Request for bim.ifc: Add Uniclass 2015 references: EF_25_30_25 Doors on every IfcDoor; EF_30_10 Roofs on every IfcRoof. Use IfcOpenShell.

First a look at what the model holds.

```python
import ifcopenshell

model = ifcopenshell.open("bim.ifc")
print(model.schema)
print("classifications:", [c.Name for c in model.by_type("IfcClassification")])
for ifc_class in ("IfcDoor", "IfcRoof", "IfcStair", "IfcWall", "IfcWindow"):
    print(ifc_class, len(model.by_type(ifc_class)))
```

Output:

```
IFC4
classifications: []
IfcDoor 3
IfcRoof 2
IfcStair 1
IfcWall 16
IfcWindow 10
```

```python
import ifcopenshell
import ifcopenshell.api.classification

model = ifcopenshell.open("bim.ifc")

system = ifcopenshell.api.classification.add_classification(model, classification="Uniclass 2015")

codes = {
    "IfcDoor": ("EF_25_30_25", "Doors"),
    "IfcRoof": ("EF_30_10", "Roofs"),
}
for ifc_class, (code, name) in codes.items():
    products = model.by_type(ifc_class)
    ifcopenshell.api.classification.add_reference(
        model, products=products, classification=system, identification=code, name=name
    )
    print(code, len(products))

model.write("bim-out.ifc")
```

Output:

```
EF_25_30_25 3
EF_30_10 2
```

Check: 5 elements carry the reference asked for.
